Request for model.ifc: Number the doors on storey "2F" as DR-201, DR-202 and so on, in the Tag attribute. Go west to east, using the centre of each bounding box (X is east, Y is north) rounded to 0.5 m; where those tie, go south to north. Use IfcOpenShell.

First a look at what the model holds.

```python
import ifcopenshell
import ifcopenshell.util.element
import ifcopenshell.util.placement

model = ifcopenshell.open("model.ifc")
print(model.schema)
storey = next(s for s in model.by_type("IfcBuildingStorey") if s.Name == "2F")
doors = [e for e in ifcopenshell.util.element.get_decomposition(storey) if e.is_a("IfcDoor")]
for e in sorted(doors, key=lambda e: e.id()):
    origin = ifcopenshell.util.placement.get_local_placement(e.ObjectPlacement)[:3, 3]
    print(e.id(), e.Tag, e.Name, origin.round(2) + 0.0, sep=" | ")
```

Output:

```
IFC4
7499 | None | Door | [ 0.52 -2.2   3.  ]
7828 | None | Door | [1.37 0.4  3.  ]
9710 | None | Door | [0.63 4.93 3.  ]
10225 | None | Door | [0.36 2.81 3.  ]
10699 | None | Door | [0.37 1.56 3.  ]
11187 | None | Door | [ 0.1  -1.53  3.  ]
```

```python
import ifcopenshell
import ifcopenshell.geom
import ifcopenshell.util.element
import ifcopenshell.util.shape

model = ifcopenshell.open("model.ifc")
settings = ifcopenshell.geom.settings()
settings.set("use-world-coords", True)


def centre(element):
    shape = ifcopenshell.geom.create_shape(settings, element)
    return ifcopenshell.util.shape.get_bbox_centroid(shape.geometry)


storey = next(s for s in model.by_type("IfcBuildingStorey") if s.Name == "2F")
doors = [e for e in ifcopenshell.util.element.get_decomposition(storey) if e.is_a("IfcDoor")]

# Insertion points can sit at a corner or the storey origin, so sort by the geometry (in metres).
centres = {e: centre(e) for e in doors}
doors.sort(key=lambda e: (round(centres[e][0] / 0.5), centres[e][1]))

for i, e in enumerate(doors, start=1):
    number = f"DR-2{i:02d}"
    e.Tag = number
    print(e.id(), number)

model.write("model-out.ifc")
```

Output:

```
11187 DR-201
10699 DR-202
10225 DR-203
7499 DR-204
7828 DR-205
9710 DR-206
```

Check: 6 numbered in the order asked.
